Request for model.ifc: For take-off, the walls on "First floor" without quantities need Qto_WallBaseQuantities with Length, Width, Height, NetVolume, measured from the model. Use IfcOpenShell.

First a look at what the model holds.

```python
import ifcopenshell
import ifcopenshell.util.element
import ifcopenshell.util.unit

model = ifcopenshell.open("model.ifc")
print(model.schema)
for unit_type in ("LENGTHUNIT", "AREAUNIT", "VOLUMEUNIT"):
    print(unit_type, ifcopenshell.util.unit.calculate_unit_scale(model, unit_type))
storey = next(s for s in model.by_type("IfcBuildingStorey") if s.Name == "First floor")
walls = [e for e in ifcopenshell.util.element.get_decomposition(storey) if e.is_a("IfcWall")]
for e in sorted(walls, key=lambda e: e.id()):
    print(e.id(), e.is_a(), e.Name, list(ifcopenshell.util.element.get_psets(e, qtos_only=True)), sep=" | ")
```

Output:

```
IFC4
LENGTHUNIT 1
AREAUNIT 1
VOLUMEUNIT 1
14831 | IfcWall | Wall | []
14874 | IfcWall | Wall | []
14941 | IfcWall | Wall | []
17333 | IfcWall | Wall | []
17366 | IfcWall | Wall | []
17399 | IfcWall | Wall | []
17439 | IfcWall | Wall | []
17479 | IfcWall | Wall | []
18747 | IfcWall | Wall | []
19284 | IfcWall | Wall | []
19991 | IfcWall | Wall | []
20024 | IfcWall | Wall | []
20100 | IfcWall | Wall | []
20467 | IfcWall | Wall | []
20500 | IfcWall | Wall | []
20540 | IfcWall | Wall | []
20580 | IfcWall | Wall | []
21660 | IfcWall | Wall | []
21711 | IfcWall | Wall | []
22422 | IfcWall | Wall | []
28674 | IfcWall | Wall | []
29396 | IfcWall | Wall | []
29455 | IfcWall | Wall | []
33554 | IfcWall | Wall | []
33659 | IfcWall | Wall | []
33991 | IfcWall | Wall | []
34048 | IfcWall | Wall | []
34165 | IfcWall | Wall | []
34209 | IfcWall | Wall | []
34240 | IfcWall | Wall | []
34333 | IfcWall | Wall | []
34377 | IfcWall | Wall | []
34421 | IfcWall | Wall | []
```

```python
import ifcopenshell
import ifcopenshell.api.pset
import ifcopenshell.geom
import ifcopenshell.util.element
import ifcopenshell.util.shape
import ifcopenshell.util.unit

model = ifcopenshell.open("model.ifc")
unit_scale = ifcopenshell.util.unit.calculate_unit_scale(model)
volume_scale = ifcopenshell.util.unit.calculate_unit_scale(model, "VOLUMEUNIT")
settings = ifcopenshell.geom.settings()

storey = next(s for s in model.by_type("IfcBuildingStorey") if s.Name == "First floor")
walls = [e for e in ifcopenshell.util.element.get_decomposition(storey) if e.is_a("IfcWall")]

for e in sorted(walls, key=lambda e: e.id()):
    if ifcopenshell.util.element.get_psets(e, qtos_only=True, should_inherit=False):
        continue
    # Geometry comes back in metres, in the element's own axes.
    shape = ifcopenshell.geom.create_shape(settings, e)
    values = {
        "Length": ifcopenshell.util.shape.get_x(shape.geometry) / unit_scale,
        "Width": ifcopenshell.util.shape.get_y(shape.geometry) / unit_scale,
        "Height": ifcopenshell.util.shape.get_z(shape.geometry) / unit_scale,
        "NetVolume": ifcopenshell.util.shape.get_volume(shape.geometry) / volume_scale,
    }
    qto = ifcopenshell.api.pset.add_qto(model, product=e, name="Qto_WallBaseQuantities")
    ifcopenshell.api.pset.edit_qto(model, qto=qto, properties=values)
    print(e.id(), {k: round(v, 3) for k, v in values.items()})

model.write("model_v2.ifc")
```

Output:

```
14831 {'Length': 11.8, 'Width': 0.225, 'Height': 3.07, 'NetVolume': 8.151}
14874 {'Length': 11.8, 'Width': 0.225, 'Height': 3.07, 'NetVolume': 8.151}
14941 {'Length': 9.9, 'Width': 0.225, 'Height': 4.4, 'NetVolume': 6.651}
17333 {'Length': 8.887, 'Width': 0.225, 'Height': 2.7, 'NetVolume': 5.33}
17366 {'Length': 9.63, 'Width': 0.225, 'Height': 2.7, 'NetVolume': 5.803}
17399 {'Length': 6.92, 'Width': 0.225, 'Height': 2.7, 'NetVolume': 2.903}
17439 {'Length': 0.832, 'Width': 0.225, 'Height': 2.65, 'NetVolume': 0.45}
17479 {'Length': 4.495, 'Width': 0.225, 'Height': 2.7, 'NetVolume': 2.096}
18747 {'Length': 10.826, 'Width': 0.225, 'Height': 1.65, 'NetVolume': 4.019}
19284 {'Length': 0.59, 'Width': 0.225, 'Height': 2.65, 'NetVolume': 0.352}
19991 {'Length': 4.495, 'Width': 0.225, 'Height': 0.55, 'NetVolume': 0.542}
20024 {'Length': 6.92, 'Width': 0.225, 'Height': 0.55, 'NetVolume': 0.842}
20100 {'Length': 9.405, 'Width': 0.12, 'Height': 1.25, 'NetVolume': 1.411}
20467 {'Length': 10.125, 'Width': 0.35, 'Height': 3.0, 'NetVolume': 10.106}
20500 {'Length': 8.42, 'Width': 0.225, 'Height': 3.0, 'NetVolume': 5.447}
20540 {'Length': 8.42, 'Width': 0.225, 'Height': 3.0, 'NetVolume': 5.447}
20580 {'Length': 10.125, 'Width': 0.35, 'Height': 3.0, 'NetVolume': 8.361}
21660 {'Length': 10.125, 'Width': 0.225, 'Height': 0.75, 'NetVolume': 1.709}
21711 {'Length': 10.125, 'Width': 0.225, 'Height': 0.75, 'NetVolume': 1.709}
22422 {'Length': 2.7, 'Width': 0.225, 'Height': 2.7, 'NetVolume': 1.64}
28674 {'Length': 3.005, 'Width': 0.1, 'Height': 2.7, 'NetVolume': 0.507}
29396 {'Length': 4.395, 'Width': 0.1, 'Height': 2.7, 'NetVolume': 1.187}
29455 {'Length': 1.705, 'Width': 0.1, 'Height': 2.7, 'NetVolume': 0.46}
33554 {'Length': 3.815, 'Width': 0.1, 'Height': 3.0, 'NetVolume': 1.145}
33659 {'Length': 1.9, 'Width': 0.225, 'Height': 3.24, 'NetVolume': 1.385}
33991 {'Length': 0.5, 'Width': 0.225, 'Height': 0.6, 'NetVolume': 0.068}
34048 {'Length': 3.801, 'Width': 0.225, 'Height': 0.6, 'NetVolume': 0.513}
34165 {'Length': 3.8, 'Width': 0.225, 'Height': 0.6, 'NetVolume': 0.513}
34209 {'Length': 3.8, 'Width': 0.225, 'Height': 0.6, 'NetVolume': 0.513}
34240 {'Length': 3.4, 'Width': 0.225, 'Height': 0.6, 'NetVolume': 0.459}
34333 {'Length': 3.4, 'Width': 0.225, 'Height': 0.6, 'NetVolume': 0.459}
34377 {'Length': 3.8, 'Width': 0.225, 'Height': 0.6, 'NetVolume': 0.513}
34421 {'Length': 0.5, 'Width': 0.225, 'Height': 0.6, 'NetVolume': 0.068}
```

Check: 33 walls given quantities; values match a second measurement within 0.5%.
